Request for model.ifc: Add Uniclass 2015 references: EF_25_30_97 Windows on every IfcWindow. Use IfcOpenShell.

First a look at what the model holds.

```python
import ifcopenshell

model = ifcopenshell.open("model.ifc")
print(model.schema)
print("classifications:", [c.Name for c in model.by_type("IfcClassification")])
for ifc_class in ("IfcDoor", "IfcRoof", "IfcStair", "IfcWall", "IfcWindow"):
    print(ifc_class, len(model.by_type(ifc_class)))
```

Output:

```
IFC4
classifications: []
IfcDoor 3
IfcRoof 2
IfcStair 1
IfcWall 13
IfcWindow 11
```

```python
import ifcopenshell
import ifcopenshell.api.classification

model = ifcopenshell.open("model.ifc")

system = ifcopenshell.api.classification.add_classification(model, classification="Uniclass 2015")

codes = {
    "IfcWindow": ("EF_25_30_97", "Windows"),
}
for ifc_class, (code, name) in codes.items():
    products = model.by_type(ifc_class)
    ifcopenshell.api.classification.add_reference(
        model, products=products, classification=system, identification=code, name=name
    )
    print(code, len(products))

model.write("model_v2.ifc")
```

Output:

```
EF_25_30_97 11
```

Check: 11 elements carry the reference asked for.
